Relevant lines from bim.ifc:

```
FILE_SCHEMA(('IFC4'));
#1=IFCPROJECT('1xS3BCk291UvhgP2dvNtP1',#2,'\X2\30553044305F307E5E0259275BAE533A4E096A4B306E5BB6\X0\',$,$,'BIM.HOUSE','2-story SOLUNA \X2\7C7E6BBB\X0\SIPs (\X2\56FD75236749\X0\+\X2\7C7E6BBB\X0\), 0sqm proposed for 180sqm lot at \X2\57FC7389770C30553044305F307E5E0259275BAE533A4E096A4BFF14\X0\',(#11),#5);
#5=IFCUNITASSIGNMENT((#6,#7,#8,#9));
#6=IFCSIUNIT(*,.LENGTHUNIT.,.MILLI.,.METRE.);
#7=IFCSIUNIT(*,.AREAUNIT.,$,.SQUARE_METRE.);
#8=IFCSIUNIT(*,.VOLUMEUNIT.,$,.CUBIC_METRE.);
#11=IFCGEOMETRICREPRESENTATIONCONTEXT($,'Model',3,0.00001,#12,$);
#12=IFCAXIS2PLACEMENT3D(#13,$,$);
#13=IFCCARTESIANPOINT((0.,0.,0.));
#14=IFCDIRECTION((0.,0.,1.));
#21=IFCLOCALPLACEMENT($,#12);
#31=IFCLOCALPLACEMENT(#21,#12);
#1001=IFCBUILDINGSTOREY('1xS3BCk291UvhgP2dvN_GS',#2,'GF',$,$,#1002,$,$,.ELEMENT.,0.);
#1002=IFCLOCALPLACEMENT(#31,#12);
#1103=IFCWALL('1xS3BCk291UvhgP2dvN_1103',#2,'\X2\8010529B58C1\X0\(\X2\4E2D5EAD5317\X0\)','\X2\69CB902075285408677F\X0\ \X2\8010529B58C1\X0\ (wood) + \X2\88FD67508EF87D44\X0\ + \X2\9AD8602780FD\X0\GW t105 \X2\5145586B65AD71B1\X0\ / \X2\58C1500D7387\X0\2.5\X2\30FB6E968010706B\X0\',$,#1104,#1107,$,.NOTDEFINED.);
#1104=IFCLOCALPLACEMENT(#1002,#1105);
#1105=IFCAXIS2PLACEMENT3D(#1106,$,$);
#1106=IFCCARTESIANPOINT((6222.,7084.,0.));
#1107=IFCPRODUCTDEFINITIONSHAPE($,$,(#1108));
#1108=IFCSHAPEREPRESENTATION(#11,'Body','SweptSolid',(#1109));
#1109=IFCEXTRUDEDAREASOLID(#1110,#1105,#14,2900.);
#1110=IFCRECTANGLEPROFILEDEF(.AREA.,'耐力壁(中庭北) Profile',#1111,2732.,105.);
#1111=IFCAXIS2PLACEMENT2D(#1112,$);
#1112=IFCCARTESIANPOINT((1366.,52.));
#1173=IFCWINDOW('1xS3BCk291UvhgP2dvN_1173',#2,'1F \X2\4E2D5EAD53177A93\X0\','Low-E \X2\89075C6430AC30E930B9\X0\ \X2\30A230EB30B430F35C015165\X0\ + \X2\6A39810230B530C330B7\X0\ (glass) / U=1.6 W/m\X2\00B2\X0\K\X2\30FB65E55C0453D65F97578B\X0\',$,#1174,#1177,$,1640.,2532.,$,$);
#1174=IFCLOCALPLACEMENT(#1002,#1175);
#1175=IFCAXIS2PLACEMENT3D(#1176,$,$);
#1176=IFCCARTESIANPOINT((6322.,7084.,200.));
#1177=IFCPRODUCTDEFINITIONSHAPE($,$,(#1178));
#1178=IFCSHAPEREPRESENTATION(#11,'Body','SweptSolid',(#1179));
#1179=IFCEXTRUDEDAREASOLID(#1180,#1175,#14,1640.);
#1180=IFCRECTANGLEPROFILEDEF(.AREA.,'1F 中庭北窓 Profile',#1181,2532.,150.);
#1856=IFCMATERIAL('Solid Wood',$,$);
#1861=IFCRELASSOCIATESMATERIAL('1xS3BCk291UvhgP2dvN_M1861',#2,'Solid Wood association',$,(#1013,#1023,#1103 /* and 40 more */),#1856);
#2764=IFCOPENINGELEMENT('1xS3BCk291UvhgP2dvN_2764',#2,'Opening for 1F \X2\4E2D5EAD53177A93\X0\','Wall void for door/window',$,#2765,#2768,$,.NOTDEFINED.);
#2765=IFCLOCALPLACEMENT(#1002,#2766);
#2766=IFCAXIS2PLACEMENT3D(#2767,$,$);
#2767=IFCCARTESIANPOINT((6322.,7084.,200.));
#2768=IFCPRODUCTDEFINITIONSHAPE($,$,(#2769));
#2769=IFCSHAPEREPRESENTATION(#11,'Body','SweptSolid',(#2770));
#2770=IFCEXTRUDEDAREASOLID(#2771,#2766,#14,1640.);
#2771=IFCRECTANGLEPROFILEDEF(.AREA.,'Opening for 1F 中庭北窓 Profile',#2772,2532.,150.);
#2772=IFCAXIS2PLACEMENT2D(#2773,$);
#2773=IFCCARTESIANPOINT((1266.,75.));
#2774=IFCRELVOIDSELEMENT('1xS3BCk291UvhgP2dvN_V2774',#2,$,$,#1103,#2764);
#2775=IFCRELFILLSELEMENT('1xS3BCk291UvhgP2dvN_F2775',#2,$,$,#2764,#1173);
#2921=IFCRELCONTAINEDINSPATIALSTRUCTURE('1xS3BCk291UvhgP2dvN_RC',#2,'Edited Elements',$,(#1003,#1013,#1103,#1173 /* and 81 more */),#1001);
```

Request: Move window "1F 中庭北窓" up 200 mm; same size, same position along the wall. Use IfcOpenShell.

```python
import numpy as np
import ifcopenshell
import ifcopenshell.api.geometry
import ifcopenshell.util.placement
import ifcopenshell.util.unit

model = ifcopenshell.open("bim.ifc")
unit_scale = ifcopenshell.util.unit.calculate_unit_scale(model)

window = model.by_id(1173)
opening = window.FillsVoids[0].RelatingOpeningElement
dz = 200.0

shift = np.array([0.0, 0.0, dz])
# The window is not placed relative to its opening, so move both.
for product in (opening, window):
    matrix = ifcopenshell.util.placement.get_local_placement(product.ObjectPlacement)
    matrix[:3, 3] += shift
    ifcopenshell.api.geometry.edit_object_placement(model, product=product, matrix=matrix, is_si=False)

print(f"moved by {dz * unit_scale:+.3f} m")

model.write("bim-out.ifc")
```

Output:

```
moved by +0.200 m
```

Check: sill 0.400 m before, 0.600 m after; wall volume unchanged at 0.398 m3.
